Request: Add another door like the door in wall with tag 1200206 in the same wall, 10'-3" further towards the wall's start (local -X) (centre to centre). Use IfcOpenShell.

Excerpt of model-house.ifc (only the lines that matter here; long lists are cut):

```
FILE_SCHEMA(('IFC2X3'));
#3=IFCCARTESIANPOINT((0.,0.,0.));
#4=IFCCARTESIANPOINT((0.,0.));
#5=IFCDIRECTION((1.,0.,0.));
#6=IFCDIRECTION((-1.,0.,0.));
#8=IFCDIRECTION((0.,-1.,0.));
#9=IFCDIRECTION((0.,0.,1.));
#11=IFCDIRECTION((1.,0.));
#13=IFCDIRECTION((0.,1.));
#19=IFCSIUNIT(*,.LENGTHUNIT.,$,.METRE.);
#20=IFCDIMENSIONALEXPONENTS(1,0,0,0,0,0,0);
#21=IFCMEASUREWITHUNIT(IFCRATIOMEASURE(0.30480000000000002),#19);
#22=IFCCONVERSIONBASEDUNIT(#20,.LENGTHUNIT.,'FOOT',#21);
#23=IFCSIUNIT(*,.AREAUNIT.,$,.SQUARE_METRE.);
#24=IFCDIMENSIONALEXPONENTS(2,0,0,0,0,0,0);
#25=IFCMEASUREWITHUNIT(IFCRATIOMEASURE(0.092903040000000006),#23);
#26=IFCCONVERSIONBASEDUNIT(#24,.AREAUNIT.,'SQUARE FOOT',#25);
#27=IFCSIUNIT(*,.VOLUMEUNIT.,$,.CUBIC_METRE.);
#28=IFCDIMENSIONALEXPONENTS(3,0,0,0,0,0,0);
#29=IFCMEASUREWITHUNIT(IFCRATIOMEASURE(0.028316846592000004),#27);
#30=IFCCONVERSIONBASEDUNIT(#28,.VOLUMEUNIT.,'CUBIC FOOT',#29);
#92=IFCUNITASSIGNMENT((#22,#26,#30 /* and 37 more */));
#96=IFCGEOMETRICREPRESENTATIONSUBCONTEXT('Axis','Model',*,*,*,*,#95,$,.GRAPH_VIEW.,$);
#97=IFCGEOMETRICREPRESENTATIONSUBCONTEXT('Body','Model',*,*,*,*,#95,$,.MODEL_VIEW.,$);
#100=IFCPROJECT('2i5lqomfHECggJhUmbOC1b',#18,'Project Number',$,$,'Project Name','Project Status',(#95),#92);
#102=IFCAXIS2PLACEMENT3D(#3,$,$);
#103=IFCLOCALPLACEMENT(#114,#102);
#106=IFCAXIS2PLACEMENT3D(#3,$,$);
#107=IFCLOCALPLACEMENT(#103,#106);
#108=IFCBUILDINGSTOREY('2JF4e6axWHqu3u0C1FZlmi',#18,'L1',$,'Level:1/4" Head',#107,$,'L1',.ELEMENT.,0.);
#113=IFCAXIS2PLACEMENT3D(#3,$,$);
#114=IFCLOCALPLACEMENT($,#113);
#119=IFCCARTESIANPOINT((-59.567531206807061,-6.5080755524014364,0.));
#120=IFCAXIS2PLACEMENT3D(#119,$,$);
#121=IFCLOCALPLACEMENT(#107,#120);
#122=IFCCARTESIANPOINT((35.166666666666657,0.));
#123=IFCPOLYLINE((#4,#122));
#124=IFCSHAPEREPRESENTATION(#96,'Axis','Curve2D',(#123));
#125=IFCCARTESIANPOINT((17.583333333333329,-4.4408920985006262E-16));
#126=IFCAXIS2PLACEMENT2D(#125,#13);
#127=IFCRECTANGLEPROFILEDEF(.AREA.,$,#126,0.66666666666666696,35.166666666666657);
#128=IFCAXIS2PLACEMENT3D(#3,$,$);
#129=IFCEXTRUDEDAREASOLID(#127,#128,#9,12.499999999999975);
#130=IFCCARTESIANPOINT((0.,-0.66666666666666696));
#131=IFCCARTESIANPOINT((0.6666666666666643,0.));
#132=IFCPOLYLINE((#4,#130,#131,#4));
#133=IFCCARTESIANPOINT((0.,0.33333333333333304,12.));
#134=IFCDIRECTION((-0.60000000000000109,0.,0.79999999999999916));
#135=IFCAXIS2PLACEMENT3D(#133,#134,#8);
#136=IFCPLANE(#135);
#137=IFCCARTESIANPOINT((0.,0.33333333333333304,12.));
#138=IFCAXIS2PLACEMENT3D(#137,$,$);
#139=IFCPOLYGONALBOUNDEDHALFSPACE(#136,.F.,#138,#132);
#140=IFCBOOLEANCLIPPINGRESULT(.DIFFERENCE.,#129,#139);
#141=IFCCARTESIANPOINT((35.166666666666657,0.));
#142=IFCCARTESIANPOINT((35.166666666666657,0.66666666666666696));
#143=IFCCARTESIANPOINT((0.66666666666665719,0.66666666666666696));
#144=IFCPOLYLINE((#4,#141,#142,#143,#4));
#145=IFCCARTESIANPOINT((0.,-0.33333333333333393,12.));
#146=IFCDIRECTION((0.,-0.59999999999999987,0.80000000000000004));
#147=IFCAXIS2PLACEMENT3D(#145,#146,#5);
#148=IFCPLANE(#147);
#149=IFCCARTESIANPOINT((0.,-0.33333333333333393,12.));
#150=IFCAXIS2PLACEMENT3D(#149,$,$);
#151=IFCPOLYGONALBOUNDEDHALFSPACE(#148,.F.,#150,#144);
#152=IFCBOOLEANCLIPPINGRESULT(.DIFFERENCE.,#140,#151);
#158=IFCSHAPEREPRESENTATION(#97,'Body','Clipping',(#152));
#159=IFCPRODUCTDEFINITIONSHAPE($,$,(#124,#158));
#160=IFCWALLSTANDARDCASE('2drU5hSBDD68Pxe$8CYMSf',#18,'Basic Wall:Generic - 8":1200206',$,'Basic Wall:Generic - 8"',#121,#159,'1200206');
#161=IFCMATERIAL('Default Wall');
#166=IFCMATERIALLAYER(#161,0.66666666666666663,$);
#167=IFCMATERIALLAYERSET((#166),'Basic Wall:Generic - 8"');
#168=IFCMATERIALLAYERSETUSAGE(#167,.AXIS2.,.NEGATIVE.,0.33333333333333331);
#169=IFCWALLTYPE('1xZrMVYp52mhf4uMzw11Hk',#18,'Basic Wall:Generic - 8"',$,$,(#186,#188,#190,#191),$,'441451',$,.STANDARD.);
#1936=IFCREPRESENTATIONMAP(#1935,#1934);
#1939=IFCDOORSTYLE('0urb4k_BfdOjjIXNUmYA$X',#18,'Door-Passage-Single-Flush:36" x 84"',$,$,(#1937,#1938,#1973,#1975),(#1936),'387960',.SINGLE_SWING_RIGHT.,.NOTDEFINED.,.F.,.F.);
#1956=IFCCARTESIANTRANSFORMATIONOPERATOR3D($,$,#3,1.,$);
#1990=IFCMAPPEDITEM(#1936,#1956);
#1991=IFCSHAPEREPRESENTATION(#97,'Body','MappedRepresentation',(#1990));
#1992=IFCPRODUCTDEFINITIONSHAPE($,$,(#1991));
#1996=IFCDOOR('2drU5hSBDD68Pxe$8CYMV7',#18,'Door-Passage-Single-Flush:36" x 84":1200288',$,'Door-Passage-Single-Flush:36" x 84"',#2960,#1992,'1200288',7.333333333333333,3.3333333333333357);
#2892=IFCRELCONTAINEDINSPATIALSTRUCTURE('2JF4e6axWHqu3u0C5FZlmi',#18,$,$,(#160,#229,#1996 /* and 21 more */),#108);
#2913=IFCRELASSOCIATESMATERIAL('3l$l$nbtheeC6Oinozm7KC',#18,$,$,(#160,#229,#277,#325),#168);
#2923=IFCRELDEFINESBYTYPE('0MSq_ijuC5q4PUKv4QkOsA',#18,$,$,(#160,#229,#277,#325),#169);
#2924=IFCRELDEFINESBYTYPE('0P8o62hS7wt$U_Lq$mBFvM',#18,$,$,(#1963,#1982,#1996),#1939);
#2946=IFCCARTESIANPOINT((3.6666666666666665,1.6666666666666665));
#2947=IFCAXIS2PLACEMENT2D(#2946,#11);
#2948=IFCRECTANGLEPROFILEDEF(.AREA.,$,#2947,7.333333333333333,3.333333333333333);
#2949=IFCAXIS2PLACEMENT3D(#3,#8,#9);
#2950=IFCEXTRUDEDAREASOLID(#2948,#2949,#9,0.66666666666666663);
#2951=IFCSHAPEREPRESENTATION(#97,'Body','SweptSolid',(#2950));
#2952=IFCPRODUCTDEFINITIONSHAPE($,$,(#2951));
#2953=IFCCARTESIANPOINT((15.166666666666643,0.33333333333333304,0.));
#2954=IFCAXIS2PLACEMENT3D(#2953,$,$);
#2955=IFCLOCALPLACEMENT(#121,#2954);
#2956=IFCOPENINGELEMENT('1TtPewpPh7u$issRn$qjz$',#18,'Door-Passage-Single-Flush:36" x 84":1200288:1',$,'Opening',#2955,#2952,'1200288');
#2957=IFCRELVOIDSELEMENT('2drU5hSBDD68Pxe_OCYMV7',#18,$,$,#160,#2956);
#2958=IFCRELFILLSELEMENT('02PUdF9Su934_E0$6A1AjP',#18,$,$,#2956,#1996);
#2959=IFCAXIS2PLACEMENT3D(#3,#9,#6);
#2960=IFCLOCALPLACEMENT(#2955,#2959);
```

```python
import ifcopenshell
import ifcopenshell.api.feature
import ifcopenshell.api.geometry
import ifcopenshell.api.root
import ifcopenshell.geom
import ifcopenshell.util.element
import ifcopenshell.util.placement
import ifcopenshell.util.shape
import ifcopenshell.util.unit

model = ifcopenshell.open("model-house.ifc")
unit_scale = ifcopenshell.util.unit.calculate_unit_scale(model)
settings = ifcopenshell.geom.settings()


def volume(element):
    """Net volume in cubic metres, openings subtracted."""
    shape = ifcopenshell.geom.create_shape(settings, element)
    return ifcopenshell.util.shape.get_volume(shape.geometry)


def reuse_history(source, copy):
    """copy_class also copies each property set's owner history, people and application; keep the originals."""
    for rel in copy.IsDefinedBy:
        if rel.is_a("IfcRelDefinesByProperties") and (history := rel.RelatingPropertyDefinition.OwnerHistory):
            rel.RelatingPropertyDefinition.OwnerHistory = source.OwnerHistory
            ifcopenshell.util.element.remove_deep2(model, history)


door = model.by_guid("2drU5hSBDD68Pxe$8CYMV7")
opening = door.FillsVoids[0].RelatingOpeningElement
wall = opening.VoidsElements[0].RelatingBuildingElement
before = volume(wall)
shift = ifcopenshell.util.placement.get_local_placement(wall.ObjectPlacement)[:3, 0] * -123 * 0.0254 / unit_scale

# copy_class copies the void relationship, type, container and properties, but no geometry.
new_opening = ifcopenshell.api.root.copy_class(model, product=opening)
new_opening.Representation = ifcopenshell.util.element.copy_deep(
    model, opening.Representation, exclude=["IfcGeometricRepresentationContext", "IfcRepresentationMap"]
)
new_opening.Name = 'Door-Passage-Single-Flush:36" x 84"'
new_opening.Tag = None
new_door = ifcopenshell.api.root.copy_class(model, product=door)
new_door.Representation = ifcopenshell.util.element.copy_deep(
    model, door.Representation, exclude=["IfcGeometricRepresentationContext", "IfcRepresentationMap"]
)
new_door.Name = 'Door-Passage-Single-Flush:36" x 84"'
new_door.Tag = None
reuse_history(door, new_door)
fills = ifcopenshell.api.feature.add_filling(model, opening=new_opening, element=new_door)
fills.OwnerHistory = new_door.OwnerHistory  # required in IFC2X3

for old, new in ((opening, new_opening), (door, new_door)):
    matrix = ifcopenshell.util.placement.get_local_placement(old.ObjectPlacement)
    matrix[:3, 3] += shift
    ifcopenshell.api.geometry.edit_object_placement(model, product=new, matrix=matrix, is_si=False)

after = volume(wall)

print(f"wall volume {before:.3f} -> {after:.3f} m3")

model.write("model-house_v2.ifc")
```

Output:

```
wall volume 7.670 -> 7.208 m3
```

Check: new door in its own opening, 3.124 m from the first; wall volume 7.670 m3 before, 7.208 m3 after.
